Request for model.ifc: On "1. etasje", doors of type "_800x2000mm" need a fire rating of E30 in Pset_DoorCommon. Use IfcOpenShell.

First a look at what the model holds.

```python
import ifcopenshell
import ifcopenshell.util.element

model = ifcopenshell.open("model.ifc")
print(model.schema)
storey = next(s for s in model.by_type("IfcBuildingStorey") if s.Name == "1. etasje")
doors = [e for e in ifcopenshell.util.element.get_decomposition(storey) if e.is_a("IfcDoor")]
seen = {}
for e in doors:
    element_type = ifcopenshell.util.element.get_type(e)
    key = (element_type.Name if element_type != e and element_type else None, ifcopenshell.util.element.get_pset(e, "Pset_DoorCommon", "FireRating"))
    seen[key] = seen.get(key, 0) + 1
for (name, value), count in sorted(seen.items(), key=str):
    print(count, "x", name, "|", value)
```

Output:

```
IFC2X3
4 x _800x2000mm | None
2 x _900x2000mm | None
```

```python
import ifcopenshell
import ifcopenshell.api.pset
import ifcopenshell.util.element

model = ifcopenshell.open("model.ifc")

storey = next(s for s in model.by_type("IfcBuildingStorey") if s.Name == "1. etasje")
doors = [e for e in ifcopenshell.util.element.get_decomposition(storey) if e.is_a("IfcDoor")]

count = 0
for e in doors:
    element_type = ifcopenshell.util.element.get_type(e)
    if element_type in (None, e) or element_type.Name != "_800x2000mm":
        continue
    # add_pset returns the element's existing set when there is one.
    pset = ifcopenshell.api.pset.add_pset(model, product=e, name="Pset_DoorCommon")
    ifcopenshell.api.pset.edit_pset(model, pset=pset, properties={"FireRating": "E30"})
    count += 1

print(count, "doors updated")

model.write("model_v2.ifc")
```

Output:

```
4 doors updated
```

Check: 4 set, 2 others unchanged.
